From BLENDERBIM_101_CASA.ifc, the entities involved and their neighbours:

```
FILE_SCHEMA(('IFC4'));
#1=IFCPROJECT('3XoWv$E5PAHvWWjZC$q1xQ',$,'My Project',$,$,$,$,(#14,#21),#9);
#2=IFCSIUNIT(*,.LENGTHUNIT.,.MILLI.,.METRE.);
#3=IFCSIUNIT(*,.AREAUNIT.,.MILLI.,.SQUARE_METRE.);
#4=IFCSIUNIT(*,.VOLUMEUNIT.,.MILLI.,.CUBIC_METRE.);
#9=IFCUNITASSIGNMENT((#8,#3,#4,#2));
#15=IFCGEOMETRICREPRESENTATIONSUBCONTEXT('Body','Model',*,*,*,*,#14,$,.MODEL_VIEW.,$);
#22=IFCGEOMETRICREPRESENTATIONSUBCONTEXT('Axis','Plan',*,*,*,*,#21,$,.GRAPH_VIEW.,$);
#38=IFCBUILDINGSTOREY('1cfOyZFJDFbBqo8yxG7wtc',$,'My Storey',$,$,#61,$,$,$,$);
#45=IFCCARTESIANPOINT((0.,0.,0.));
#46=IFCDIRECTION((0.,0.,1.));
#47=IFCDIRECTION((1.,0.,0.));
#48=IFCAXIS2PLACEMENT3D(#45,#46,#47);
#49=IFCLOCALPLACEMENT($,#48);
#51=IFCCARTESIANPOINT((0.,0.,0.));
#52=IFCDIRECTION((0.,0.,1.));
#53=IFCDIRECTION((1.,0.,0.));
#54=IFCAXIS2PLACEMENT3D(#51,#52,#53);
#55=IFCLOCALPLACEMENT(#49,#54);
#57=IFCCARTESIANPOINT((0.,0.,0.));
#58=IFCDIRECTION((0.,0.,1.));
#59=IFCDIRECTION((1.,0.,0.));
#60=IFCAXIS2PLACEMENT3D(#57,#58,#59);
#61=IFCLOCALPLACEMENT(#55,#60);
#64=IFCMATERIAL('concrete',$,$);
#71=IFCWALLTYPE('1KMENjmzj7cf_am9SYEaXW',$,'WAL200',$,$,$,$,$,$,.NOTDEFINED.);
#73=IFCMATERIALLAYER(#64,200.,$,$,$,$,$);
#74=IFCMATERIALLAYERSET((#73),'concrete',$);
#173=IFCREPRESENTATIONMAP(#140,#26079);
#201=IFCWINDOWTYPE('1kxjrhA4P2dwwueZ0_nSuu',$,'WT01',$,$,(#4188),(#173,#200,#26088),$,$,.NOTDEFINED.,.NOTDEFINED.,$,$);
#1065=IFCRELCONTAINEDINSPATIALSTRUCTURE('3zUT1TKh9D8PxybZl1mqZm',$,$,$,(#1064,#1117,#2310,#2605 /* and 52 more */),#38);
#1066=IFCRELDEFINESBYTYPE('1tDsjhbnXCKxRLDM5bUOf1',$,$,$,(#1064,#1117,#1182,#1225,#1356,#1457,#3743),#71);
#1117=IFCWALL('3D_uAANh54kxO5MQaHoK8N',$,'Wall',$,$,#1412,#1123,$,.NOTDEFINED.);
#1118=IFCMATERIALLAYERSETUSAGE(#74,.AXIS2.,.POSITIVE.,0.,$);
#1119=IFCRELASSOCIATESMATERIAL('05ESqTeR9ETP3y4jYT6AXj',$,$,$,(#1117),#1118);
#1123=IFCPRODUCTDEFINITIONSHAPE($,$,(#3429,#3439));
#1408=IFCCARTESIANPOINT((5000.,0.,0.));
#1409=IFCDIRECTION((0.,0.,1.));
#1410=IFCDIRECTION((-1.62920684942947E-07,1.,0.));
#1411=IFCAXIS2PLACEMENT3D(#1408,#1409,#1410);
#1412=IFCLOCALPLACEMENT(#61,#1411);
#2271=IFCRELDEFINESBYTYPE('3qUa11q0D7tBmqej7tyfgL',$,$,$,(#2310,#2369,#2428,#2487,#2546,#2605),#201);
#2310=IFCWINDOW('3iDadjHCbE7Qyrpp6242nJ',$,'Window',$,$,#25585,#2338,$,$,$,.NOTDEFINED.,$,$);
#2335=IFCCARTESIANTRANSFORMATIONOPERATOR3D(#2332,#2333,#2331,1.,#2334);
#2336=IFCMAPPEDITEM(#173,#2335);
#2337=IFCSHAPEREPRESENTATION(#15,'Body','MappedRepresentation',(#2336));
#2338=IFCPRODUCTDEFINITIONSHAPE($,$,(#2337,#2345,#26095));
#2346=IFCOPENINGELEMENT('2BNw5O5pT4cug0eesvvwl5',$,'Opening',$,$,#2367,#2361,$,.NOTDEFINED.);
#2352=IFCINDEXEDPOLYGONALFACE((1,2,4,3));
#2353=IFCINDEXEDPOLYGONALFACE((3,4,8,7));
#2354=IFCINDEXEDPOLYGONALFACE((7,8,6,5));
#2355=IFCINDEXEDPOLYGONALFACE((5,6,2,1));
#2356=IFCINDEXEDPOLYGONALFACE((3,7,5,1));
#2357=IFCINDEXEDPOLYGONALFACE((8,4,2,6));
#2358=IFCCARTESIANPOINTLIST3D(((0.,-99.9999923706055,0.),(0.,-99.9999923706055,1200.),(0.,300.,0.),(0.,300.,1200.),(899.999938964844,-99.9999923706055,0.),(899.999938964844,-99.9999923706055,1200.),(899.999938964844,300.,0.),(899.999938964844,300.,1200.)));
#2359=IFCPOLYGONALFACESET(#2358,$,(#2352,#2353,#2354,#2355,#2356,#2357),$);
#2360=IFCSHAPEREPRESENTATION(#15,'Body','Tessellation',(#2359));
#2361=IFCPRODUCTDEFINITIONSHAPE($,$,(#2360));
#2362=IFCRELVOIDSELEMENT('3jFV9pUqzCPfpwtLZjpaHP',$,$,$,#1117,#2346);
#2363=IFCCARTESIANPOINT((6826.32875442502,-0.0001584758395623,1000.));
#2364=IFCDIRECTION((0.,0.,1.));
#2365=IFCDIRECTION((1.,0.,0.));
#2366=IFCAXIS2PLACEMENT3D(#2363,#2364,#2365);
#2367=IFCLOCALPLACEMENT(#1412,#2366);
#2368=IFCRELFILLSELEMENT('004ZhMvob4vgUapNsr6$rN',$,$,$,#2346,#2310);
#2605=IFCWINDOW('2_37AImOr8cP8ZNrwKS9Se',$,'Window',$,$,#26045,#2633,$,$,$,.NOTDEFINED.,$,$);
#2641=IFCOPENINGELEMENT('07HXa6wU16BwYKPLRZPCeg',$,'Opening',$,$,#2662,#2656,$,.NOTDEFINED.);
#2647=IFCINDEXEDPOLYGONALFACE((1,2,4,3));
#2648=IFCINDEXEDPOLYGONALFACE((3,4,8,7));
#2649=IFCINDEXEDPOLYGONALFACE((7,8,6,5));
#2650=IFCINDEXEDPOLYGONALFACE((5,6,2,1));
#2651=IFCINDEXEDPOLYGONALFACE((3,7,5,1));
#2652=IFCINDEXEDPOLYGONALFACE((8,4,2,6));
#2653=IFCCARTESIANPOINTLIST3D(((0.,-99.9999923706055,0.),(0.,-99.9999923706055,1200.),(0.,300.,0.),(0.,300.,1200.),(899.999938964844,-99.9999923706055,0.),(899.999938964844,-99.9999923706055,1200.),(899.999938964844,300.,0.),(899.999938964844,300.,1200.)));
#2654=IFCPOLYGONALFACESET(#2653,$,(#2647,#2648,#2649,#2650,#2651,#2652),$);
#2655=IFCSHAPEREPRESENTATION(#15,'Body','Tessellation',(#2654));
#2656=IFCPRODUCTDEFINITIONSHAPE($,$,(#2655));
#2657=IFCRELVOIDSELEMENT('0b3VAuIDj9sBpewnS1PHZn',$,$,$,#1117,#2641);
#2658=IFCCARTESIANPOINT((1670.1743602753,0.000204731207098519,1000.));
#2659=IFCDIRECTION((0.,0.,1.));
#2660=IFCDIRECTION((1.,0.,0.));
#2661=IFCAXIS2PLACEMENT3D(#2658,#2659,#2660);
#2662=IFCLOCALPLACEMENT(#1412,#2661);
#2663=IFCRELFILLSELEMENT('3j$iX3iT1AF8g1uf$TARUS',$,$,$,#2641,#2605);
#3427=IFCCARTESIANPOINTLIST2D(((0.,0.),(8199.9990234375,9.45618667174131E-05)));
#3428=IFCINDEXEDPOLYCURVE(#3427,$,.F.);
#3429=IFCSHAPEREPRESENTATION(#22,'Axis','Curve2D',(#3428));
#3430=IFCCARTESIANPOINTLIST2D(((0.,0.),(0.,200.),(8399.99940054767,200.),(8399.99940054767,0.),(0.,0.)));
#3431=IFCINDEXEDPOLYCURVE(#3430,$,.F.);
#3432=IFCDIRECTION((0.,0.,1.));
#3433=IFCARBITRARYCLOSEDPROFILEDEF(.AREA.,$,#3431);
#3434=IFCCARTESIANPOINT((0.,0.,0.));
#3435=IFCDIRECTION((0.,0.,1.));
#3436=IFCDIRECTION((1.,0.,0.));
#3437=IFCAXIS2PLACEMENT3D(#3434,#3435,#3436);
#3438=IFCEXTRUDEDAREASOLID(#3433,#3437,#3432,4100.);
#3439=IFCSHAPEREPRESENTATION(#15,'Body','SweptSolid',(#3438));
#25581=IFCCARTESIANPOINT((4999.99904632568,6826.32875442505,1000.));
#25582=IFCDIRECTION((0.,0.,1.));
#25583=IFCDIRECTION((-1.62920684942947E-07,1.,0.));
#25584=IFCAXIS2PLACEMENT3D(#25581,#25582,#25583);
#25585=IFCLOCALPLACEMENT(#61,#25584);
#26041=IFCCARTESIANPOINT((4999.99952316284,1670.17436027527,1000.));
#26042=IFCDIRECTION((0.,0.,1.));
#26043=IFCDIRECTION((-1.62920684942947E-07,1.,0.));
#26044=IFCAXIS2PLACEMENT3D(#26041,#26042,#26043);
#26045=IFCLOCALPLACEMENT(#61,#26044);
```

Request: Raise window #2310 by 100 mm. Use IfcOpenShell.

```python
import numpy as np
import ifcopenshell
import ifcopenshell.api.geometry
import ifcopenshell.util.placement
import ifcopenshell.util.unit

model = ifcopenshell.open("BLENDERBIM_101_CASA.ifc")
unit_scale = ifcopenshell.util.unit.calculate_unit_scale(model)

window = model.by_guid("3iDadjHCbE7Qyrpp6242nJ")
opening = window.FillsVoids[0].RelatingOpeningElement
dz = 100.0

shift = np.array([0.0, 0.0, dz])
# The window is not placed relative to its opening, so move both.
for product in (opening, window):
    matrix = ifcopenshell.util.placement.get_local_placement(product.ObjectPlacement)
    matrix[:3, 3] += shift
    ifcopenshell.api.geometry.edit_object_placement(model, product=product, matrix=matrix, is_si=False)

print(f"moved by {dz * unit_scale:+.3f} m")

model.write("BLENDERBIM_101_CASA-out.ifc")
```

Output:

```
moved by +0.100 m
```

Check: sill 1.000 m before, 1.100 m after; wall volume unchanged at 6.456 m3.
